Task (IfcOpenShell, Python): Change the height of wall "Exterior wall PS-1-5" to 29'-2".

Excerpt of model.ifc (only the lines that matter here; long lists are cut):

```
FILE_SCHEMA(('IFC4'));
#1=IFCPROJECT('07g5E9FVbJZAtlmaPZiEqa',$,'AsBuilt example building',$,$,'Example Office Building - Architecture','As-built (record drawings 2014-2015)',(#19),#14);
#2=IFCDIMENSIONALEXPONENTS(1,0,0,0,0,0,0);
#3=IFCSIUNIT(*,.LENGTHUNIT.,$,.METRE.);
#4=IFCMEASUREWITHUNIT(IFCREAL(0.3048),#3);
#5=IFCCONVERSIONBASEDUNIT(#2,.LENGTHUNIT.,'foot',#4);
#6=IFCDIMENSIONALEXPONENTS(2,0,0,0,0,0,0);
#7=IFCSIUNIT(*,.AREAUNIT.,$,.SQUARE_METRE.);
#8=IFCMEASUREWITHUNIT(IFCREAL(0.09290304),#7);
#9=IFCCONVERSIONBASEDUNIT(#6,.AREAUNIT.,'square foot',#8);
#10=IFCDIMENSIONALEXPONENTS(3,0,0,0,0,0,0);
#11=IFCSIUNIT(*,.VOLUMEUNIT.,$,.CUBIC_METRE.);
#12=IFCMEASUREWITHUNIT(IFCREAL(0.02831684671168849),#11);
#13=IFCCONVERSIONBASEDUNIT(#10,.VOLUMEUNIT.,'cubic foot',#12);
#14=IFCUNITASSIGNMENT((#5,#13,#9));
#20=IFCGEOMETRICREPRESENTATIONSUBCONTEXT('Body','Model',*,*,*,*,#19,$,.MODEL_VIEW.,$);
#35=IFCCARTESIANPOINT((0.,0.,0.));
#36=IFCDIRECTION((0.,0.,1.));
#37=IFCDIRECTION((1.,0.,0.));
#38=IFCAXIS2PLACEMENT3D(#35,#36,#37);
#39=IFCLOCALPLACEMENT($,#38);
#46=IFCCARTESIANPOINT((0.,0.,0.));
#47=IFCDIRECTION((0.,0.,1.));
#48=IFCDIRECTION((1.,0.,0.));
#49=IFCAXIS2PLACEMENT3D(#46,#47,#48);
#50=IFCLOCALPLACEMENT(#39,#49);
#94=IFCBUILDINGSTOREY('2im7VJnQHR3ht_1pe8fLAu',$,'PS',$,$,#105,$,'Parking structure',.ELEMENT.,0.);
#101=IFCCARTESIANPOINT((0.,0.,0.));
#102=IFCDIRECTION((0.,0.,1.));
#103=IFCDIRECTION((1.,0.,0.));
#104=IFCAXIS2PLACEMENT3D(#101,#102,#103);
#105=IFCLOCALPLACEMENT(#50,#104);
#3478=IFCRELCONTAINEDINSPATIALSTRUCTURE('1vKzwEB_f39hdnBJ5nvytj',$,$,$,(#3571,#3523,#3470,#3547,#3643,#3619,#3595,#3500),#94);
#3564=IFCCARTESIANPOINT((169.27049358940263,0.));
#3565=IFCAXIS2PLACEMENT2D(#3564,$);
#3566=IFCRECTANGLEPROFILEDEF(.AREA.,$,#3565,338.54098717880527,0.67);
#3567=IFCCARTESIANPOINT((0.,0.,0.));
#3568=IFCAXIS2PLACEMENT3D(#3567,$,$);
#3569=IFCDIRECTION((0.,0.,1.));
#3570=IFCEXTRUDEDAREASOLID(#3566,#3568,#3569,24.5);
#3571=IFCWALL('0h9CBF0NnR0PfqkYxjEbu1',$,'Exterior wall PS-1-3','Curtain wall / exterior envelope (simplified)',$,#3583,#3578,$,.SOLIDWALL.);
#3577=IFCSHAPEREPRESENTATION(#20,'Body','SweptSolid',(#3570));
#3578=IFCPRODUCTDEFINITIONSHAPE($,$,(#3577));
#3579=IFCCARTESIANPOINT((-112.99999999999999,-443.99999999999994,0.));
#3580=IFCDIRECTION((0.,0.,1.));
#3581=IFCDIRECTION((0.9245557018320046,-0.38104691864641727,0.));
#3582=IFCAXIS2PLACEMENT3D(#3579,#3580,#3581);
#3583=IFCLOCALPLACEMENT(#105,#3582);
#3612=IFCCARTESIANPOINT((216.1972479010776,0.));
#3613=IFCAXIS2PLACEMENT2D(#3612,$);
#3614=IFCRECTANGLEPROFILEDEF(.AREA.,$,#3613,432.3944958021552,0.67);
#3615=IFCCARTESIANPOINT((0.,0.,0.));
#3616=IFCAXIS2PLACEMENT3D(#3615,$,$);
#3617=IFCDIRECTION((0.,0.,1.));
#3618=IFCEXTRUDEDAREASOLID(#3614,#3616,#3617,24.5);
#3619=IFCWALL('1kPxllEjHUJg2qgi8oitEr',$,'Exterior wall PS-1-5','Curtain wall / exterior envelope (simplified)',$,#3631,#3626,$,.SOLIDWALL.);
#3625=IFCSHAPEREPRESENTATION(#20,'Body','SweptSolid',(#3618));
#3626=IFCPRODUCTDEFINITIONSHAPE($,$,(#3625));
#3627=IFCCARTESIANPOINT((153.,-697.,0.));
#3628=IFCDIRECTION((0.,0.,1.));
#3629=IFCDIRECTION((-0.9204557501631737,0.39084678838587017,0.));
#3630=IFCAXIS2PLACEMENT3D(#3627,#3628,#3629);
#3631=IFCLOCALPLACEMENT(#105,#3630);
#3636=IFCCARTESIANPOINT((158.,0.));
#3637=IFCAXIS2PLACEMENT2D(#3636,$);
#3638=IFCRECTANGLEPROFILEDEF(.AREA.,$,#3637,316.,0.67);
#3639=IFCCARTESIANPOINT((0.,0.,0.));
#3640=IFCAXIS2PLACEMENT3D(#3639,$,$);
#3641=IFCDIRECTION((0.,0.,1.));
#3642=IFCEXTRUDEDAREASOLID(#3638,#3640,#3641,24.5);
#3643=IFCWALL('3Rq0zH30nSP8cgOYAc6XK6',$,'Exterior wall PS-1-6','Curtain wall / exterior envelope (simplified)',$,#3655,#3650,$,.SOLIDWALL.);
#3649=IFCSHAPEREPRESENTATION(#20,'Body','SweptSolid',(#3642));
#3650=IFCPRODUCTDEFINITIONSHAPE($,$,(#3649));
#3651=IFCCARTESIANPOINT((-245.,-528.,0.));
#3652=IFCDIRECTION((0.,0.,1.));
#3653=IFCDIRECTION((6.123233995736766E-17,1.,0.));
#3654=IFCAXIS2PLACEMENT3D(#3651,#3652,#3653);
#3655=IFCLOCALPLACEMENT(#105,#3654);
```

```python
import ifcopenshell
import ifcopenshell.geom
import ifcopenshell.util.representation
import ifcopenshell.util.shape
import ifcopenshell.util.unit

model = ifcopenshell.open("model.ifc")
unit_scale = ifcopenshell.util.unit.calculate_unit_scale(model)
settings = ifcopenshell.geom.settings()


def volume(element):
    """Net volume in cubic metres, openings subtracted."""
    shape = ifcopenshell.geom.create_shape(settings, element)
    return ifcopenshell.util.shape.get_volume(shape.geometry)


wall = model.by_guid("1kPxllEjHUJg2qgi8oitEr")
before = volume(wall)

body = ifcopenshell.util.representation.get_representation(wall, "Model", "Body")
solid = body.Items[0]
old_height = solid.Depth
solid.Depth = 350 * 0.0254 / unit_scale
after = volume(wall)

print(f"height {old_height:g} -> {solid.Depth:g}, volume {before:.3f} -> {after:.3f} m3")

model.write("model_rev.ifc")
```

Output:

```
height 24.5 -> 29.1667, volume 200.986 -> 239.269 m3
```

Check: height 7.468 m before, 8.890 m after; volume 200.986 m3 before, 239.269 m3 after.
